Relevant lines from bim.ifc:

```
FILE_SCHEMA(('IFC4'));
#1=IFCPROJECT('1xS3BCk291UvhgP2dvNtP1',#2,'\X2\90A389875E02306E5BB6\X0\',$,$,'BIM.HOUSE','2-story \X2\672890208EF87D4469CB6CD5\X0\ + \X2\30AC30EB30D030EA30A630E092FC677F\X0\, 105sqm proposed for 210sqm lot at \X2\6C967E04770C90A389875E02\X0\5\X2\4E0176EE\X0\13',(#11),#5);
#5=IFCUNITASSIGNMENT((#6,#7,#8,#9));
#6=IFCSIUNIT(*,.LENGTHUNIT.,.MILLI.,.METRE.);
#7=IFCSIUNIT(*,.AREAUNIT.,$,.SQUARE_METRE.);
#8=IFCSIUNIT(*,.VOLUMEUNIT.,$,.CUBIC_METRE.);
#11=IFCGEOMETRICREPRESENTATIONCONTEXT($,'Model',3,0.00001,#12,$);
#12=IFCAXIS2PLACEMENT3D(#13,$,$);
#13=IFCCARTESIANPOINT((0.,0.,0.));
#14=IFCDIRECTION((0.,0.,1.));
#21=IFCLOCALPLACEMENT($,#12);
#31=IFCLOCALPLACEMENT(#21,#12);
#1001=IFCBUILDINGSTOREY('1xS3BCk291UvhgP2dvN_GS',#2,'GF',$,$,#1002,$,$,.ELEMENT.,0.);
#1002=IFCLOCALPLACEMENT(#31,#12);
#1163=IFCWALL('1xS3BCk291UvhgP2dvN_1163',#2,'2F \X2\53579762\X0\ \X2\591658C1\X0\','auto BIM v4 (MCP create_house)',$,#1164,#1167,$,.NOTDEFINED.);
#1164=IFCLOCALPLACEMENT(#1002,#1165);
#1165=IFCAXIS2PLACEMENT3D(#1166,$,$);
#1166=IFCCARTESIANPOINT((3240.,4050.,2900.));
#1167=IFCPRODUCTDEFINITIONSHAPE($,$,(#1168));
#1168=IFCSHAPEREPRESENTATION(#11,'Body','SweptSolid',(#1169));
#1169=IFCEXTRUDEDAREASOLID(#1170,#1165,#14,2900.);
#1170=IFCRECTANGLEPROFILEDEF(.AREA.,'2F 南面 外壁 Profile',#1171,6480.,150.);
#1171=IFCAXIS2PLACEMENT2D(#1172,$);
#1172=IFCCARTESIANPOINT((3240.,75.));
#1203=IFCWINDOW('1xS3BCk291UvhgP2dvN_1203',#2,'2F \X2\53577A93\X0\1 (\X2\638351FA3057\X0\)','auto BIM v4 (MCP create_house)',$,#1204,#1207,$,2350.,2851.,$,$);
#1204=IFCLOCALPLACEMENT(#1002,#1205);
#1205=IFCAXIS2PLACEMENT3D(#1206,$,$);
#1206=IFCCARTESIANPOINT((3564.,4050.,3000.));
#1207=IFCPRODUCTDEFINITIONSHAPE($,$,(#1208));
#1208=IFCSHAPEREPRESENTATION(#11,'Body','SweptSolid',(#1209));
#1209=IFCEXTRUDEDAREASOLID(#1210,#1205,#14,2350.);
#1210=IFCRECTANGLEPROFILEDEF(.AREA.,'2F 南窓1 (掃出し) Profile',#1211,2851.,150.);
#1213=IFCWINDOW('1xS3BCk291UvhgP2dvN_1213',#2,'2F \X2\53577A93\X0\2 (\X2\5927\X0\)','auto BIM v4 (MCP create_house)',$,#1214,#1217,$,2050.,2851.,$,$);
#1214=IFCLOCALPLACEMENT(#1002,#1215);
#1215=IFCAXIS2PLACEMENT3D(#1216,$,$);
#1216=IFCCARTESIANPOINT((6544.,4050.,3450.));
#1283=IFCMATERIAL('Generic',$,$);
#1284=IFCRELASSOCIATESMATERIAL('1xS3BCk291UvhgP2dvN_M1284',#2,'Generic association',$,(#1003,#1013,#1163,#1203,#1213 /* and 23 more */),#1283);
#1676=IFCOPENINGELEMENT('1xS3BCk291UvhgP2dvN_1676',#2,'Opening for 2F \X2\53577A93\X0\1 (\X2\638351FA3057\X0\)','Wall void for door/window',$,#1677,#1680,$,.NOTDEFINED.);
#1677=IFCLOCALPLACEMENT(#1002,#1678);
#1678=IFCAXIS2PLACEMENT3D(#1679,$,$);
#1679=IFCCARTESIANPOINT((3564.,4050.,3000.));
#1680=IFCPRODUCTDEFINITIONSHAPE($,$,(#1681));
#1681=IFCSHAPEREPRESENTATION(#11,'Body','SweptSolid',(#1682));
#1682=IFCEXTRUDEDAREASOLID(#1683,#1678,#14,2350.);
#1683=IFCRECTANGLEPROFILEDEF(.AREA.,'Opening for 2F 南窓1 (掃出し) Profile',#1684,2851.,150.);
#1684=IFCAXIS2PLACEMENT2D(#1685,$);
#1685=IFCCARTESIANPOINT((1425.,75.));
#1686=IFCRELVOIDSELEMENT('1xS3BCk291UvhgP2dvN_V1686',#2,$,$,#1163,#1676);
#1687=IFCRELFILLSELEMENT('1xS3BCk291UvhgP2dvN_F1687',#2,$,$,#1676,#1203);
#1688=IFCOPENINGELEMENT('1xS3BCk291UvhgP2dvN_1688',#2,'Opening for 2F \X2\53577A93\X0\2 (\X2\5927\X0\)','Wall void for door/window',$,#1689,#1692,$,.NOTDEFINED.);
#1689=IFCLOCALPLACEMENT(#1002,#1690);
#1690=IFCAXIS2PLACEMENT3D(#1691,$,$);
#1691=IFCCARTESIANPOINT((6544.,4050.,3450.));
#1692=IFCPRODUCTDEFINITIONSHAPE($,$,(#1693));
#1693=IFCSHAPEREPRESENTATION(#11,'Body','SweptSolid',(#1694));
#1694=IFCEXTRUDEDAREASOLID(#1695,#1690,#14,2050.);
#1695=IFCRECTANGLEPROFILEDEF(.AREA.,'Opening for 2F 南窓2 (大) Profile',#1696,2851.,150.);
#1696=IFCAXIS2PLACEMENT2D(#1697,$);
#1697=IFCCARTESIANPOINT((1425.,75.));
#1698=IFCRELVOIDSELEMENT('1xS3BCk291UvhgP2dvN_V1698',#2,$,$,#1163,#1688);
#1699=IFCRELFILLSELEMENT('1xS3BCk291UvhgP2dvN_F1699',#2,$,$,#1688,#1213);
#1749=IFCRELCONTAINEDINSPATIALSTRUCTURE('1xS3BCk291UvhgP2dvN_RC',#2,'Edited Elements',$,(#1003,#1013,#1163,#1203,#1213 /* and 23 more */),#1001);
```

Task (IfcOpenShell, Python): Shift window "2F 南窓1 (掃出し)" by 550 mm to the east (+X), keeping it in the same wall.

```python
import ifcopenshell
import ifcopenshell.api.geometry
import ifcopenshell.util.placement
import ifcopenshell.util.unit

model = ifcopenshell.open("bim.ifc")
unit_scale = ifcopenshell.util.unit.calculate_unit_scale(model)

window = model.by_guid("1xS3BCk291UvhgP2dvN_1203")
opening = window.FillsVoids[0].RelatingOpeningElement
wall = opening.VoidsElements[0].RelatingBuildingElement

wall_matrix = ifcopenshell.util.placement.get_local_placement(wall.ObjectPlacement)
shift = wall_matrix[:3, 0] * 0.55 / unit_scale
before = ifcopenshell.util.placement.get_local_placement(window.ObjectPlacement)[:3, 3].copy()

# The window is not placed relative to its opening, so move both.
for product in (opening, window):
    matrix = ifcopenshell.util.placement.get_local_placement(product.ObjectPlacement)
    matrix[:3, 3] += shift
    ifcopenshell.api.geometry.edit_object_placement(model, product=product, matrix=matrix, is_si=False)

after = ifcopenshell.util.placement.get_local_placement(window.ObjectPlacement)[:3, 3]
print("window moved by", (after - before).round(3) + 0.0)

model.write("bim_v2.ifc")
```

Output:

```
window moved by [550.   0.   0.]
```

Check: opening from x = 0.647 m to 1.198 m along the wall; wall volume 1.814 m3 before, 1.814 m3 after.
